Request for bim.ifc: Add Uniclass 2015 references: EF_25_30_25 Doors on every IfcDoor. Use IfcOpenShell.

First a look at what the model holds.

```python
import ifcopenshell

model = ifcopenshell.open("bim.ifc")
print(model.schema)
print("classifications:", [c.Name for c in model.by_type("IfcClassification")])
for ifc_class in ("IfcDoor", "IfcRoof", "IfcStair", "IfcWall", "IfcWindow"):
    print(ifc_class, len(model.by_type(ifc_class)))
```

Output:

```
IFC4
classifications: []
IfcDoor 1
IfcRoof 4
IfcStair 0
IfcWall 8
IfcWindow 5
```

```python
import ifcopenshell
import ifcopenshell.api.classification

model = ifcopenshell.open("bim.ifc")

system = ifcopenshell.api.classification.add_classification(model, classification="Uniclass 2015")

codes = {
    "IfcDoor": ("EF_25_30_25", "Doors"),
}
for ifc_class, (code, name) in codes.items():
    products = model.by_type(ifc_class)
    ifcopenshell.api.classification.add_reference(
        model, products=products, classification=system, identification=code, name=name
    )
    print(code, len(products))

model.write("bim_updated.ifc")
```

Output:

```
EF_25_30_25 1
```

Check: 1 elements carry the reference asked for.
